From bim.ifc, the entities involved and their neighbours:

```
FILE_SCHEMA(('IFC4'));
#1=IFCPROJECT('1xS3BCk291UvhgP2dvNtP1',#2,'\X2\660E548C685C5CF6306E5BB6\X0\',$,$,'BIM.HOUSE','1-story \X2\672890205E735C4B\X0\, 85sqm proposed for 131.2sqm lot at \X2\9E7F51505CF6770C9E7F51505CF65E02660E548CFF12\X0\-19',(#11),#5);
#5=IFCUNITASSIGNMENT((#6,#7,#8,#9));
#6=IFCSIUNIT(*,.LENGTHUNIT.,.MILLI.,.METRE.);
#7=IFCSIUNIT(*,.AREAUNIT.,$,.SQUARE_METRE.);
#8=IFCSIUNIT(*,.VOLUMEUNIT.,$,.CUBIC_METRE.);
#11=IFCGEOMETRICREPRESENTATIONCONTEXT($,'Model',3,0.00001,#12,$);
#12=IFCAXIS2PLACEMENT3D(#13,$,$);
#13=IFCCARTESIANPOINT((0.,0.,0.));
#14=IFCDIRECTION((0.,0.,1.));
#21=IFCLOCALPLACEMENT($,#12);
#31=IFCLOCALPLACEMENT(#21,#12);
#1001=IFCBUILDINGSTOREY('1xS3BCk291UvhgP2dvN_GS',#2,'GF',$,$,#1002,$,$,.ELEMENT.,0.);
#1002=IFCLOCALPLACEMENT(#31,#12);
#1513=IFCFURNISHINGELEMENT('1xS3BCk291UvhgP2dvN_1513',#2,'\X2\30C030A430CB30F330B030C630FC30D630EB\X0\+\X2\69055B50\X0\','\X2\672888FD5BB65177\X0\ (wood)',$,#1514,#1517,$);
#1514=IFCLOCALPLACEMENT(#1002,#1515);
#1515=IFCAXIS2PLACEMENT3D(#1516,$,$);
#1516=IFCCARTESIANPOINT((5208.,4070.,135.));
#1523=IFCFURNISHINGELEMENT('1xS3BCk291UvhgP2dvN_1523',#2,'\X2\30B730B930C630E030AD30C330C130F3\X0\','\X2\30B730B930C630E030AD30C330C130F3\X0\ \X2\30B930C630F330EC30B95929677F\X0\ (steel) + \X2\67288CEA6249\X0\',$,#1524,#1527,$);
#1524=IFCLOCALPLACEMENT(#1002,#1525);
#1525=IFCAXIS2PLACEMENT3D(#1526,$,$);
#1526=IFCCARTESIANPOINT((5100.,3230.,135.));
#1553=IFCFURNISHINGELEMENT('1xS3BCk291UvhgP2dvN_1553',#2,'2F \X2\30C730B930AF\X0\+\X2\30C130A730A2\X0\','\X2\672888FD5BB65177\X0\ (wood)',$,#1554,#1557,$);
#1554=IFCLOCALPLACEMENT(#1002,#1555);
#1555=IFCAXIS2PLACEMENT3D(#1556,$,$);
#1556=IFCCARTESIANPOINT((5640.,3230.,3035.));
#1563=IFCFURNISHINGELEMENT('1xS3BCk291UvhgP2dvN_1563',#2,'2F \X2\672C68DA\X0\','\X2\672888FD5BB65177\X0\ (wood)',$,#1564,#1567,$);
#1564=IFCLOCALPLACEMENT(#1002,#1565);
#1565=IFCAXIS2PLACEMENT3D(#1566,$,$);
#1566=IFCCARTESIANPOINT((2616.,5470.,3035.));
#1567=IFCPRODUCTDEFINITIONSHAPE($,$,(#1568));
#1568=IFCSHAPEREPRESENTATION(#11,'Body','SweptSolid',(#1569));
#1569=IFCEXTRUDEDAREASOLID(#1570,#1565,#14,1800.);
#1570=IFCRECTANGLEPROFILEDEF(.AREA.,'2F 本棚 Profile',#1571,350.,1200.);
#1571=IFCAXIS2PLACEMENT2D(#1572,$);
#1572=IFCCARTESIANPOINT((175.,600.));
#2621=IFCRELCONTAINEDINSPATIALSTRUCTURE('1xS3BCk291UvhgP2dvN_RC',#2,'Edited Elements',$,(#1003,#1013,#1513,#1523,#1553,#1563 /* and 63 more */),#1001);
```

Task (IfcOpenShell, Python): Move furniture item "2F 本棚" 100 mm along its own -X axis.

```python
import ifcopenshell
import ifcopenshell.api.geometry
import ifcopenshell.util.placement

model = ifcopenshell.open("bim.ifc")

item = model.by_guid("1xS3BCk291UvhgP2dvN_1563")
matrix = ifcopenshell.util.placement.get_local_placement(item.ObjectPlacement)
matrix[:3, 3] -= matrix[:3, 0] * 100.0
ifcopenshell.api.geometry.edit_object_placement(model, product=item, matrix=matrix, is_si=False)

print(ifcopenshell.util.placement.get_local_placement(item.ObjectPlacement).round(3) + 0.0)

model.write("bim_updated.ifc")
```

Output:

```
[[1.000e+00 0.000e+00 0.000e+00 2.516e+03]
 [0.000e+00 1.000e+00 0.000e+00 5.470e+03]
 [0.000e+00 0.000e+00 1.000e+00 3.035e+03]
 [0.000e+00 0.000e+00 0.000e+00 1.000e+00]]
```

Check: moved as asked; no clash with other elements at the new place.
